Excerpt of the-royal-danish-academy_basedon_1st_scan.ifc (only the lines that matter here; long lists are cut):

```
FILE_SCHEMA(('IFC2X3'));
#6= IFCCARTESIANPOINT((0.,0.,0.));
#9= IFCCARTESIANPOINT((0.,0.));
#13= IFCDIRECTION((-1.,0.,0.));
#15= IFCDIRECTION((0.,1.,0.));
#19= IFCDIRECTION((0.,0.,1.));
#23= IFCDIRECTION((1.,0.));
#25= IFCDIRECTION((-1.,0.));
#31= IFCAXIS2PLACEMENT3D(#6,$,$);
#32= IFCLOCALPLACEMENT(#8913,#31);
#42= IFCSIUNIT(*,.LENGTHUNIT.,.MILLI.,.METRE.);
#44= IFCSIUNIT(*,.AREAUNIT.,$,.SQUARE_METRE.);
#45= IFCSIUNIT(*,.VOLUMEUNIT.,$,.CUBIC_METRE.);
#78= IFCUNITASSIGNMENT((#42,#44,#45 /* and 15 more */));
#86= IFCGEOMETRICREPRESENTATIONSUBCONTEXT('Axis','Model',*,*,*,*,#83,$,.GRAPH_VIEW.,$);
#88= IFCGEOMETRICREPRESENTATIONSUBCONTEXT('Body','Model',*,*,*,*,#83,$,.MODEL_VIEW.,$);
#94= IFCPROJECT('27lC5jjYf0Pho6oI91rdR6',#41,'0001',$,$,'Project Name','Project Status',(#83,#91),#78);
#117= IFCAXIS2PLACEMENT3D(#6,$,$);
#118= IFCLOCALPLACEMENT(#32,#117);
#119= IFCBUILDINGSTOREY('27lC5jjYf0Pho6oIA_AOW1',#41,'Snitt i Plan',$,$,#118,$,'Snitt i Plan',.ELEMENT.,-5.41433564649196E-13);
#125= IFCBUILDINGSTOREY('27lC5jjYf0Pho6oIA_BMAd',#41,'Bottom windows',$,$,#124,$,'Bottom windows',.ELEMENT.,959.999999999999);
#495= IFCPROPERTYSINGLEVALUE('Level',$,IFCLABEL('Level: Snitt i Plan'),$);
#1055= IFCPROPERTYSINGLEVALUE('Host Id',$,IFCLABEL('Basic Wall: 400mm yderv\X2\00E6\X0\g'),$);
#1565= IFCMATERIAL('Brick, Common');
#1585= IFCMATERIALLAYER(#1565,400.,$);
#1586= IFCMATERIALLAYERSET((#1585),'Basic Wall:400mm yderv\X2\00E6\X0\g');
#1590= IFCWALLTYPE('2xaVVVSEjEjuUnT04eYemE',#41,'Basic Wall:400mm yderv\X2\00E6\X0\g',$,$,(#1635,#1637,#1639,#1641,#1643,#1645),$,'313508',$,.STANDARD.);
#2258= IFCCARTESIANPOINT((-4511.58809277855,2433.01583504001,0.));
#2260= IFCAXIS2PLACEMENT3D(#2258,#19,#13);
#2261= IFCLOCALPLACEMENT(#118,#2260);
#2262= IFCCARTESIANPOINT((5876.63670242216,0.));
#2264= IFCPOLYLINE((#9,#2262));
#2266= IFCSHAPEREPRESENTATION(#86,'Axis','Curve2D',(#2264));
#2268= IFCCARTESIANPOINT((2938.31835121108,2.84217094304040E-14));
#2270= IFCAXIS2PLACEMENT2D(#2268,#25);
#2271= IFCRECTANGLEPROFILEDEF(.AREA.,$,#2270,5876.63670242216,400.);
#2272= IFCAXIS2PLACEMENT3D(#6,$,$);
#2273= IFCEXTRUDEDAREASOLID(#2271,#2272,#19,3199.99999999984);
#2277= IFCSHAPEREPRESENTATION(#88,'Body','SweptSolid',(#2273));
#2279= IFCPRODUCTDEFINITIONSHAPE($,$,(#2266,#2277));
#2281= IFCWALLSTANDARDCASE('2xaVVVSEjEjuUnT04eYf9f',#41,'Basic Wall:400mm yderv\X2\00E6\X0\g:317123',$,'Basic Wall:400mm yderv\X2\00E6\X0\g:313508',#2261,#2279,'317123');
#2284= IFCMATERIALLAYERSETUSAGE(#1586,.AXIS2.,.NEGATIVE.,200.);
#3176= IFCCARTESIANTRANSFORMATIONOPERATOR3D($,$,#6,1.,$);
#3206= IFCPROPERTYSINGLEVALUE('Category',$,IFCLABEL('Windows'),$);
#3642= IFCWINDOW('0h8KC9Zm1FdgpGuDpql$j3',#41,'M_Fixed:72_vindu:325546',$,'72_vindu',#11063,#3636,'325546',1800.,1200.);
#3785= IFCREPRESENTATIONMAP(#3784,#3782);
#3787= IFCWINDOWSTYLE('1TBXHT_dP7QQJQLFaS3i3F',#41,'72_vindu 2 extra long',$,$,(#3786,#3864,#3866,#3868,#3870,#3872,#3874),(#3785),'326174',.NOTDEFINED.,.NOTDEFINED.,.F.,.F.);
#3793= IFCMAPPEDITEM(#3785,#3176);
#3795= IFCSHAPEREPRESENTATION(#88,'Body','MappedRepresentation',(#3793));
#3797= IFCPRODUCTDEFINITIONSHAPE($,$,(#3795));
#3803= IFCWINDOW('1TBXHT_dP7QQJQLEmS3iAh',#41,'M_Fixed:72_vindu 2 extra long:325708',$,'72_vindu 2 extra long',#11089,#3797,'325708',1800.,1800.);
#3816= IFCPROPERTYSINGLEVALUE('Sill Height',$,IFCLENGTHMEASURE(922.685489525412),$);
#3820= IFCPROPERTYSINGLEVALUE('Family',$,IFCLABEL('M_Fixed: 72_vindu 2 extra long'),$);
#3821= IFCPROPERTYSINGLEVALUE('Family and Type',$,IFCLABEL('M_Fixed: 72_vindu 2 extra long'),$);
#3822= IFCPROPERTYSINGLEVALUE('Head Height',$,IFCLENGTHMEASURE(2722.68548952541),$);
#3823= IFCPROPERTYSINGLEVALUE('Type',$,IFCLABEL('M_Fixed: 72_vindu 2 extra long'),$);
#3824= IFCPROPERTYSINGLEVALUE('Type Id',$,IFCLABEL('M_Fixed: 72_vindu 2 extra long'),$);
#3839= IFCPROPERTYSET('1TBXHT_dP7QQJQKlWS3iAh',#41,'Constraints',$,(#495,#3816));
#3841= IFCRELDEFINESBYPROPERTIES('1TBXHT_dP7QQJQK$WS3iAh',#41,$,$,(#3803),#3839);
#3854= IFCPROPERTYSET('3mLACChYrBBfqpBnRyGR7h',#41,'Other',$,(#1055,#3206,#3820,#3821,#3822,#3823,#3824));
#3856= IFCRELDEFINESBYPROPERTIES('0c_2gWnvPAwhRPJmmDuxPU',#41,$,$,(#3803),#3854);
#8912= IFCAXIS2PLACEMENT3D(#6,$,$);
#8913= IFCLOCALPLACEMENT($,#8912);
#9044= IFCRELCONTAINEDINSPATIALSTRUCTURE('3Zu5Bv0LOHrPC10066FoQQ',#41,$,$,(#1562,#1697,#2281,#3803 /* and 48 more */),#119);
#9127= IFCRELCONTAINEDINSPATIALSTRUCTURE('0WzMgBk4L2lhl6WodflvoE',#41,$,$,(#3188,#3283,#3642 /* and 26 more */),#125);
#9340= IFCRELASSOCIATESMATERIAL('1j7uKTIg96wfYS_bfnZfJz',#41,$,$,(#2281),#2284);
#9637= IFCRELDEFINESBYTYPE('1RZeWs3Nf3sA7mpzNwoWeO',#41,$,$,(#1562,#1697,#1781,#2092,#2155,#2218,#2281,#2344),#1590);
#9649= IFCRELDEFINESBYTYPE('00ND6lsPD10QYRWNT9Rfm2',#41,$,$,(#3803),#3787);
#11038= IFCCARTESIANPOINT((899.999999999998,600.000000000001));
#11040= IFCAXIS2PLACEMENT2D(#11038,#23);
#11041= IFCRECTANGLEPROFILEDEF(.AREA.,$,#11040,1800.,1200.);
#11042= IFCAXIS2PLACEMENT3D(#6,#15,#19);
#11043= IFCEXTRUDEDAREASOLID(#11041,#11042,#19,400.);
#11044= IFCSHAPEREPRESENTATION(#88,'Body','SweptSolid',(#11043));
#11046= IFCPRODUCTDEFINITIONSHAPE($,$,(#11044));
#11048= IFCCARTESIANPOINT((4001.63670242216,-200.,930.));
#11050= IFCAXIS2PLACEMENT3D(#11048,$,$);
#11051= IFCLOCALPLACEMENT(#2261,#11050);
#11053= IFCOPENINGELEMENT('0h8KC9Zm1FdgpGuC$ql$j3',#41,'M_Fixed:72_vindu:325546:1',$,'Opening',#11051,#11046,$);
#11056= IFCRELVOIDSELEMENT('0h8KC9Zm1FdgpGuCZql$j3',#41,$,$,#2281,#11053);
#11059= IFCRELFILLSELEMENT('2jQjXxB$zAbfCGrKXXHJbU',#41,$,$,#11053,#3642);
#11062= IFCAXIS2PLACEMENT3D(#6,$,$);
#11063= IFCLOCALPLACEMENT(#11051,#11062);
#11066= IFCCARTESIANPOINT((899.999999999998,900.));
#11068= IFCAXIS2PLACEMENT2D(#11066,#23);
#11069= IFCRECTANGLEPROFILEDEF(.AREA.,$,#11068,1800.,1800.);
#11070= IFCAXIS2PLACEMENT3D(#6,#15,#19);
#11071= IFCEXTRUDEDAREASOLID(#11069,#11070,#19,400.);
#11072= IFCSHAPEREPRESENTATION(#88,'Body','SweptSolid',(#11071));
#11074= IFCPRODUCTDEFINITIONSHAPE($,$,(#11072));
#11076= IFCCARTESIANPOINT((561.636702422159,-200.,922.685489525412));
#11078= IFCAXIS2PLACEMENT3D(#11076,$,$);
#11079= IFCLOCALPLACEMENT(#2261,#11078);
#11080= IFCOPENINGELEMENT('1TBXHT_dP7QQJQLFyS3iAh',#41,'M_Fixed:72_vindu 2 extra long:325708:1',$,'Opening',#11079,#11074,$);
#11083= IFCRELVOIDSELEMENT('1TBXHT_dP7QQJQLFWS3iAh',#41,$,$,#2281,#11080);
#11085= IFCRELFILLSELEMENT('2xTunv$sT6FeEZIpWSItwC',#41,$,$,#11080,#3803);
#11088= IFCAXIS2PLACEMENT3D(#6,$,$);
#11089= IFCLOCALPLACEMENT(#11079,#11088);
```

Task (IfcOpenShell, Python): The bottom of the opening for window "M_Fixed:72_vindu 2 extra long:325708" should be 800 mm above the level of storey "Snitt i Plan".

```python
import numpy as np
import ifcopenshell
import ifcopenshell.api.geometry
import ifcopenshell.api.pset
import ifcopenshell.geom
import ifcopenshell.util.element
import ifcopenshell.util.placement
import ifcopenshell.util.shape
import ifcopenshell.util.unit

model = ifcopenshell.open("the-royal-danish-academy_basedon_1st_scan.ifc")
unit_scale = ifcopenshell.util.unit.calculate_unit_scale(model)

window = model.by_guid("1TBXHT_dP7QQJQLEmS3iAh")
opening = window.FillsVoids[0].RelatingOpeningElement
storey = ifcopenshell.util.element.get_container(window, ifc_class="IfcBuildingStorey")
level = ifcopenshell.util.placement.get_local_placement(storey.ObjectPlacement)[2, 3]

# The opening's origin need not be at the sill, so measure its lowest point.
shape = ifcopenshell.geom.create_shape(ifcopenshell.geom.settings(), opening)
bottom = ifcopenshell.util.shape.get_shape_bottom_elevation(shape, shape.geometry) / unit_scale
dz = level + 0.8 / unit_scale - bottom

shift = np.array([0.0, 0.0, dz])
# The window is placed relative to its opening, so it follows when the opening moves.
matrix = ifcopenshell.util.placement.get_local_placement(opening.ObjectPlacement)
matrix[:3, 3] += shift
ifcopenshell.api.geometry.edit_object_placement(
    model, product=opening, matrix=matrix, is_si=False, should_transform_children=True
)

# Keep the stored heights in step.
pset = model.by_id(ifcopenshell.util.element.get_pset(window, "Constraints", should_inherit=False)["id"])
ifcopenshell.api.pset.edit_pset(model, pset=pset, properties={
    "Sill Height": model.create_entity("IfcLengthMeasure", ifcopenshell.util.element.get_pset(window, "Constraints", "Sill Height") + dz),
})
pset = model.by_id(ifcopenshell.util.element.get_pset(window, "Other", should_inherit=False)["id"])
ifcopenshell.api.pset.edit_pset(model, pset=pset, properties={
    "Head Height": model.create_entity("IfcLengthMeasure", ifcopenshell.util.element.get_pset(window, "Other", "Head Height") + dz),
})

print(f"moved by {dz * unit_scale:+.3f} m")

model.write("the-royal-danish-academy_basedon_1st_scan_updated.ifc")
```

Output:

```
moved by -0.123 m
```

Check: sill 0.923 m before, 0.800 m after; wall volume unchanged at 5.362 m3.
